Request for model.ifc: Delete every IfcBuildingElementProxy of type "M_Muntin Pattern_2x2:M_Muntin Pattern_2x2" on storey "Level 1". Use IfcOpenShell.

First a look at what the model holds.

```python
import ifcopenshell
import ifcopenshell.util.element

model = ifcopenshell.open("model.ifc")
print(model.schema)
storey = next(s for s in model.by_type("IfcBuildingStorey") if s.Name == "Level 1")
proxies = [e for e in ifcopenshell.util.element.get_decomposition(storey) if e.is_a("IfcBuildingElementProxy")]
seen = {}
for e in proxies:
    element_type = ifcopenshell.util.element.get_type(e)
    name = element_type.Name if element_type not in (None, e) else None
    seen[name] = seen.get(name, 0) + 1
for name, count in sorted(seen.items(), key=str):
    print(count, "x", name)
```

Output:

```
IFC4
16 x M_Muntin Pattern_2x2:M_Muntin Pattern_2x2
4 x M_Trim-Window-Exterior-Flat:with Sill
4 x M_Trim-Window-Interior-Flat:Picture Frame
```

```python
import ifcopenshell
import ifcopenshell.api.root
import ifcopenshell.util.element

model = ifcopenshell.open("model.ifc")

storey = next(s for s in model.by_type("IfcBuildingStorey") if s.Name == "Level 1")
proxies = [e for e in ifcopenshell.util.element.get_decomposition(storey) if e.is_a("IfcBuildingElementProxy")]
targets = [e for e in proxies if (t := ifcopenshell.util.element.get_type(e)) not in (None, e) and t.Name == "M_Muntin Pattern_2x2:M_Muntin Pattern_2x2"]

for e in targets:
    ifcopenshell.api.root.remove_product(model, product=e)
print(len(targets), "removed")

model.write("model_updated.ifc")
```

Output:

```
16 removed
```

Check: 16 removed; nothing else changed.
